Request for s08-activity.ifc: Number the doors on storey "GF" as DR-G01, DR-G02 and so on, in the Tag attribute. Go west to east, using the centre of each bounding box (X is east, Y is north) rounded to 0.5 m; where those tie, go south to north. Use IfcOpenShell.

First a look at what the model holds.

```python
import ifcopenshell
import ifcopenshell.util.element
import ifcopenshell.util.placement

model = ifcopenshell.open("s08-activity.ifc")
print(model.schema)
storey = next(s for s in model.by_type("IfcBuildingStorey") if s.Name == "GF")
doors = [e for e in ifcopenshell.util.element.get_decomposition(storey) if e.is_a("IfcDoor")]
for e in sorted(doors, key=lambda e: e.id()):
    origin = ifcopenshell.util.placement.get_local_placement(e.ObjectPlacement)[:3, 3]
    print(e.id(), e.Tag, e.Name, origin.round(2) + 0.0, sep=" | ")
```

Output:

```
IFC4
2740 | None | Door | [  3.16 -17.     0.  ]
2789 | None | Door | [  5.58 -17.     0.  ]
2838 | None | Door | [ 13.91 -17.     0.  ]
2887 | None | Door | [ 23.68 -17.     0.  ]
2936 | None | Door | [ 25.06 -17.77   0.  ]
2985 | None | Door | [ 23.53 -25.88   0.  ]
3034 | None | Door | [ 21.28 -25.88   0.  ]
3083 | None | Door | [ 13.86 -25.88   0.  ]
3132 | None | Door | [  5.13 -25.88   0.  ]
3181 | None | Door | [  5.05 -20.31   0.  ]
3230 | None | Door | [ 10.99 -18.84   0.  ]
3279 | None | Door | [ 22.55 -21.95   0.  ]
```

```python
import ifcopenshell
import ifcopenshell.geom
import ifcopenshell.util.element
import ifcopenshell.util.shape

model = ifcopenshell.open("s08-activity.ifc")
settings = ifcopenshell.geom.settings()
settings.set("use-world-coords", True)


def centre(element):
    shape = ifcopenshell.geom.create_shape(settings, element)
    return ifcopenshell.util.shape.get_bbox_centroid(shape.geometry)


storey = next(s for s in model.by_type("IfcBuildingStorey") if s.Name == "GF")
doors = [e for e in ifcopenshell.util.element.get_decomposition(storey) if e.is_a("IfcDoor")]

# Insertion points can sit at a corner or the storey origin, so sort by the geometry (in metres).
centres = {e: centre(e) for e in doors}
doors.sort(key=lambda e: (round(centres[e][0] / 0.5), centres[e][1]))

for i, e in enumerate(doors, start=1):
    number = f"DR-G{i:02d}"
    e.Tag = number
    print(e.id(), number)

model.write("s08-activity_v2.ifc")
```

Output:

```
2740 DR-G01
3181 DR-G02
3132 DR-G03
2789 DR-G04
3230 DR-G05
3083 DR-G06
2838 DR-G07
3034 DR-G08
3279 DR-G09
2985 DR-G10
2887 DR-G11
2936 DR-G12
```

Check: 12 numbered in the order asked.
